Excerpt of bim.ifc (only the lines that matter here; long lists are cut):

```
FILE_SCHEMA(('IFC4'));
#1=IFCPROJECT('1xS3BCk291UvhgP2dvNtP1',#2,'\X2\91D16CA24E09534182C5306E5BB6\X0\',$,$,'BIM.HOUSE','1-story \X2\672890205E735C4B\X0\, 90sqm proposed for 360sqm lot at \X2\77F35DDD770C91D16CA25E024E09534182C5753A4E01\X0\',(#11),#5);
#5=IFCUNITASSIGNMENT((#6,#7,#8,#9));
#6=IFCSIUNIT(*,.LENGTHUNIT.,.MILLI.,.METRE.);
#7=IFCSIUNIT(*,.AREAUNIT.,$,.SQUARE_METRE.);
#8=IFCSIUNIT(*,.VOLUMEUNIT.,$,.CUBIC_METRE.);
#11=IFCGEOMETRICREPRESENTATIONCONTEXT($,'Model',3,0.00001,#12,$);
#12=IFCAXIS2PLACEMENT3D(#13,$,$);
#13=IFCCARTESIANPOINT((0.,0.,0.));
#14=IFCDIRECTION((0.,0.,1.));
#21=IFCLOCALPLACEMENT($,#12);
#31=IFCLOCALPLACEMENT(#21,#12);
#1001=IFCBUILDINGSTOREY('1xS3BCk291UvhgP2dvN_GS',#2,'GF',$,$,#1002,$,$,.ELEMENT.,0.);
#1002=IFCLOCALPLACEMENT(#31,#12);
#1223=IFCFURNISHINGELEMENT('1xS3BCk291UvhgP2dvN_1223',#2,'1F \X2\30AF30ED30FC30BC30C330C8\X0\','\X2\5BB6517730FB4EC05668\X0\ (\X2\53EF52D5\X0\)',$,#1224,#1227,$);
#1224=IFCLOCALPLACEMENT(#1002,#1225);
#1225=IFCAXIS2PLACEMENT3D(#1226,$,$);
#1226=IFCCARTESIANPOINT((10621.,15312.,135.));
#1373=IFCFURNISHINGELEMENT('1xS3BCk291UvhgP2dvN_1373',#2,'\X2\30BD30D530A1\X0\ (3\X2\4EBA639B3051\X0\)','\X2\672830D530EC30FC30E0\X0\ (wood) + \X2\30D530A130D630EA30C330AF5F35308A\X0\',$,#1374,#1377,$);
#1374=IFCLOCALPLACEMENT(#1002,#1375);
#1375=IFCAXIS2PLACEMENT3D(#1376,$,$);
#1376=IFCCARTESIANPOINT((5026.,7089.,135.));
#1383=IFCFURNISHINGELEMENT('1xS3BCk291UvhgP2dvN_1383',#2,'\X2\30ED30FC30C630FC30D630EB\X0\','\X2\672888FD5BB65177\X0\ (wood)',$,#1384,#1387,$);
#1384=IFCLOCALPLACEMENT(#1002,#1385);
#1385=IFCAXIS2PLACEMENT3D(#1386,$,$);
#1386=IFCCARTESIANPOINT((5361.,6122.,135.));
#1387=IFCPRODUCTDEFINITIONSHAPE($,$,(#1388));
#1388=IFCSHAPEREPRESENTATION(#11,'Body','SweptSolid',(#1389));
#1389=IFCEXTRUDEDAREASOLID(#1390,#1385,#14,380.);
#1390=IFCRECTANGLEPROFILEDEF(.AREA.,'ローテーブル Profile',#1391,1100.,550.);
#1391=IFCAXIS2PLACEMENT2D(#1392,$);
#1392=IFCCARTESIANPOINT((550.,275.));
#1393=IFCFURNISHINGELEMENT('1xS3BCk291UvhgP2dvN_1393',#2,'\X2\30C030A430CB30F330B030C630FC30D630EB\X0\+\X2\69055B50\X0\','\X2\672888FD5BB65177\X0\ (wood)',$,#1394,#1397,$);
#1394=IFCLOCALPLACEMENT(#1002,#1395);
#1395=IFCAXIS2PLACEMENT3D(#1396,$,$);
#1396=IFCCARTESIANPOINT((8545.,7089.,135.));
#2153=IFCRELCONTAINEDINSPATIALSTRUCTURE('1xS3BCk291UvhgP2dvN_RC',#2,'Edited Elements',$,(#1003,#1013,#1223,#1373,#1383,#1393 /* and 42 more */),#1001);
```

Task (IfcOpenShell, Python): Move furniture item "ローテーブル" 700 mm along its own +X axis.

```python
import ifcopenshell
import ifcopenshell.api.geometry
import ifcopenshell.util.placement
import ifcopenshell.util.unit

model = ifcopenshell.open("bim.ifc")
unit_scale = ifcopenshell.util.unit.calculate_unit_scale(model)

item = model.by_id(1383)
matrix = ifcopenshell.util.placement.get_local_placement(item.ObjectPlacement)
matrix[:3, 3] += matrix[:3, 0] * 0.7 / unit_scale
ifcopenshell.api.geometry.edit_object_placement(model, product=item, matrix=matrix, is_si=False)

print(ifcopenshell.util.placement.get_local_placement(item.ObjectPlacement).round(3) + 0.0)

model.write("bim_edited.ifc")
```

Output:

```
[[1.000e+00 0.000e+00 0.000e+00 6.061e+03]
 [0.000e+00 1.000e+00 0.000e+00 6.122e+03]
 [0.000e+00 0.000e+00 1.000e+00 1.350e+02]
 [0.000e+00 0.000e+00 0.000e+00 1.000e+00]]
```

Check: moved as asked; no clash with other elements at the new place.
